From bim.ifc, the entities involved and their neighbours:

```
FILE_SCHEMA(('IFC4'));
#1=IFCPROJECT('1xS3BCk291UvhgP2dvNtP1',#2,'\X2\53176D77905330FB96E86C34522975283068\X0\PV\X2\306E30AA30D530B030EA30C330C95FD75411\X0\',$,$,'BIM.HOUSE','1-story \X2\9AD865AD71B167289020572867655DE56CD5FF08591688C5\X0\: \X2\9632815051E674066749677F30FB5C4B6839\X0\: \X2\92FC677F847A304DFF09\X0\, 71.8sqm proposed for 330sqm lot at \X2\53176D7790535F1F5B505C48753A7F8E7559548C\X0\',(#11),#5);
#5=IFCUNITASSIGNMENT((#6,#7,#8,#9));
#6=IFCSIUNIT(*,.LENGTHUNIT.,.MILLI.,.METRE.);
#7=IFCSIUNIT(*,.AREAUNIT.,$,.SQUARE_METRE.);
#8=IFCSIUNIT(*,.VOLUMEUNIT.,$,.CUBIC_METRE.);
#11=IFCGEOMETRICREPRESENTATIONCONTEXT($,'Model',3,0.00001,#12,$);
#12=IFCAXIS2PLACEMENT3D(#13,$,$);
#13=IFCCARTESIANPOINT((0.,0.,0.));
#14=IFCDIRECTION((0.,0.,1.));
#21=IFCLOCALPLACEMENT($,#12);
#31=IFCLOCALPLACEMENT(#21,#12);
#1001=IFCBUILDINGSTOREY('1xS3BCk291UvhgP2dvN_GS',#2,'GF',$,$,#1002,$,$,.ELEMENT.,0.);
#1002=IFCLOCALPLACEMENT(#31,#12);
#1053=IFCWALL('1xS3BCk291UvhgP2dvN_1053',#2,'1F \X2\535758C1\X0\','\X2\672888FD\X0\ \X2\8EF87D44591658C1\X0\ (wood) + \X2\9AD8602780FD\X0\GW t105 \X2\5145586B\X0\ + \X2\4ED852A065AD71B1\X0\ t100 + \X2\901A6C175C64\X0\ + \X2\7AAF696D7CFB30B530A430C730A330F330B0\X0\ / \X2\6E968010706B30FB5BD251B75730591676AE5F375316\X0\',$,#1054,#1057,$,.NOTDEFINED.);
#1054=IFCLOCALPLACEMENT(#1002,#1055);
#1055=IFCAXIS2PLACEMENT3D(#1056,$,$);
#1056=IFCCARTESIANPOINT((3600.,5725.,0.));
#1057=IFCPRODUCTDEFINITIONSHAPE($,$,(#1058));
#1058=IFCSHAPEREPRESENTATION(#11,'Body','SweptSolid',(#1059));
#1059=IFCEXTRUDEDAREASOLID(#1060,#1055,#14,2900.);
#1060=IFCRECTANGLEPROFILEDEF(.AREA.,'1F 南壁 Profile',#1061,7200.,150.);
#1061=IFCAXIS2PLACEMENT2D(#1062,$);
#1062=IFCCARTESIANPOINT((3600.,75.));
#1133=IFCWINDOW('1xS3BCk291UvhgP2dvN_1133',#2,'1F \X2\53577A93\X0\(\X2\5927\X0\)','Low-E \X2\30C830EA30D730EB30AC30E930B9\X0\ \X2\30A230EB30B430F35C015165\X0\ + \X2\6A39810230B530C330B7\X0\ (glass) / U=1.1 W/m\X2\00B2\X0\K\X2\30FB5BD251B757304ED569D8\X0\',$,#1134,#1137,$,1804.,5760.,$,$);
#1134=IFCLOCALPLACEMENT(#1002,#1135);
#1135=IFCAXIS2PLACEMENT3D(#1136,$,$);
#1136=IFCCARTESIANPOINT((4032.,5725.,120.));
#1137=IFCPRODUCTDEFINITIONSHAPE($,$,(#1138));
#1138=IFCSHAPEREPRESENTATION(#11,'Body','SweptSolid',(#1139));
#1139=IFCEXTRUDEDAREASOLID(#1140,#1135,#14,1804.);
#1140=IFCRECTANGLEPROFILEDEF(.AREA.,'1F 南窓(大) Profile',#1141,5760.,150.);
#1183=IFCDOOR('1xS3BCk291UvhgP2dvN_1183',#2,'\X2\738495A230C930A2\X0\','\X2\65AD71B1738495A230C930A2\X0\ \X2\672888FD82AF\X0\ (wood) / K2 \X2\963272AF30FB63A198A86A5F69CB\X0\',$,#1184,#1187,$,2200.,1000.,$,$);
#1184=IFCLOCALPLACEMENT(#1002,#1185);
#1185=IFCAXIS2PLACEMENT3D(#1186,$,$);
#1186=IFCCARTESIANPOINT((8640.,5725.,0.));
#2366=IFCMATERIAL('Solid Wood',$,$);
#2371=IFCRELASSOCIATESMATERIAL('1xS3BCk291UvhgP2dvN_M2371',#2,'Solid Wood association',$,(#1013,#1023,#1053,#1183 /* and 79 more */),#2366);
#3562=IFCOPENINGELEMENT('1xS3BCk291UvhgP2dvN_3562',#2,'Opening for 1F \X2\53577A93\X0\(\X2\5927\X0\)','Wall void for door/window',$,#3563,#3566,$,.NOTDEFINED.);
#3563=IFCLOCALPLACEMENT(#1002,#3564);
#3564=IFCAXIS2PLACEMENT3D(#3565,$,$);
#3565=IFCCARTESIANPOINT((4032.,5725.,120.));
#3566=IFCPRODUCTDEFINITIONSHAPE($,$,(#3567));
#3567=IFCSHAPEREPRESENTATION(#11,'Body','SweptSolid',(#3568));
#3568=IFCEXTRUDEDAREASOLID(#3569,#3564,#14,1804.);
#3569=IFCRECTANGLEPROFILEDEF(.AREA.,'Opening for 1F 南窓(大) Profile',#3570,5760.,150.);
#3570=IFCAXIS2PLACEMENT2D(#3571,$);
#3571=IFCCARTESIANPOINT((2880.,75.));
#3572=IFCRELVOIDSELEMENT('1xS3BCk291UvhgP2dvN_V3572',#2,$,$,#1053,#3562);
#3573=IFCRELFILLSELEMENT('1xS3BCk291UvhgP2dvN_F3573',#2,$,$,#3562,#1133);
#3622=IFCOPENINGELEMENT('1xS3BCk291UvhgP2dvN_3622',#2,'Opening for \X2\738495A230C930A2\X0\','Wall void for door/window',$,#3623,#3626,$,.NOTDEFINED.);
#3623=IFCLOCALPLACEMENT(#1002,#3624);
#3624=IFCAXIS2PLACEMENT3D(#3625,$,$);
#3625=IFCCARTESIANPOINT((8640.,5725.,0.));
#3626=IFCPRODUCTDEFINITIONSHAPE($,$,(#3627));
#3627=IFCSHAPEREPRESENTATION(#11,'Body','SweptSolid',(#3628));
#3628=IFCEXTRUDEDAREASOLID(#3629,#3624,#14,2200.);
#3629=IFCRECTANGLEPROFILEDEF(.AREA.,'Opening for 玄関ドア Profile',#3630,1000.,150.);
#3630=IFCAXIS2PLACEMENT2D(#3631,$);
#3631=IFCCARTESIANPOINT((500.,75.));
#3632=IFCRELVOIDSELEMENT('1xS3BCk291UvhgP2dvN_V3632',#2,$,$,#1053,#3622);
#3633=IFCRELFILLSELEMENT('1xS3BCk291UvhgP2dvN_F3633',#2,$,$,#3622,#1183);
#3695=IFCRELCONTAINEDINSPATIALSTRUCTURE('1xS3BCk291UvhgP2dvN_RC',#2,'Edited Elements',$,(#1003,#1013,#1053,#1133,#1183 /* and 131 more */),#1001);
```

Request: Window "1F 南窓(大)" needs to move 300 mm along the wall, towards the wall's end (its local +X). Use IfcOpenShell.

```python
import ifcopenshell
import ifcopenshell.api.geometry
import ifcopenshell.util.placement
import ifcopenshell.util.unit

model = ifcopenshell.open("bim.ifc")
unit_scale = ifcopenshell.util.unit.calculate_unit_scale(model)

window = model.by_guid("1xS3BCk291UvhgP2dvN_1133")
opening = window.FillsVoids[0].RelatingOpeningElement
wall = opening.VoidsElements[0].RelatingBuildingElement

wall_matrix = ifcopenshell.util.placement.get_local_placement(wall.ObjectPlacement)
shift = wall_matrix[:3, 0] * 0.3 / unit_scale
before = ifcopenshell.util.placement.get_local_placement(window.ObjectPlacement)[:3, 3].copy()

# The window is not placed relative to its opening, so move both.
for product in (opening, window):
    matrix = ifcopenshell.util.placement.get_local_placement(product.ObjectPlacement)
    matrix[:3, 3] += shift
    ifcopenshell.api.geometry.edit_object_placement(model, product=product, matrix=matrix, is_si=False)

after = ifcopenshell.util.placement.get_local_placement(window.ObjectPlacement)[:3, 3]
print("window moved by", (after - before).round(3) + 0.0)

model.write("bim_updated.ifc")
```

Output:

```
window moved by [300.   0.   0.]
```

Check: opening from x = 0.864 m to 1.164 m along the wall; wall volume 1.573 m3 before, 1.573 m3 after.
